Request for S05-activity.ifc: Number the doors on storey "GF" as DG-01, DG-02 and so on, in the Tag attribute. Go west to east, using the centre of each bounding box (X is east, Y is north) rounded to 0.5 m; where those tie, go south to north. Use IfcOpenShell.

First a look at what the model holds.

```python
import ifcopenshell
import ifcopenshell.util.element
import ifcopenshell.util.placement

model = ifcopenshell.open("S05-activity.ifc")
print(model.schema)
storey = next(s for s in model.by_type("IfcBuildingStorey") if s.Name == "GF")
doors = [e for e in ifcopenshell.util.element.get_decomposition(storey) if e.is_a("IfcDoor")]
for e in sorted(doors, key=lambda e: e.id()):
    origin = ifcopenshell.util.placement.get_local_placement(e.ObjectPlacement)[:3, 3]
    print(e.id(), e.Tag, e.Name, origin.round(2) + 0.0, sep=" | ")
```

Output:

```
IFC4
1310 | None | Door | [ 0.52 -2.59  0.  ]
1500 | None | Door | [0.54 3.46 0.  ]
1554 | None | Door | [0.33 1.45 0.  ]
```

```python
import ifcopenshell
import ifcopenshell.geom
import ifcopenshell.util.element
import ifcopenshell.util.shape

model = ifcopenshell.open("S05-activity.ifc")
settings = ifcopenshell.geom.settings()
settings.set("use-world-coords", True)


def centre(element):
    shape = ifcopenshell.geom.create_shape(settings, element)
    return ifcopenshell.util.shape.get_bbox_centroid(shape.geometry)


storey = next(s for s in model.by_type("IfcBuildingStorey") if s.Name == "GF")
doors = [e for e in ifcopenshell.util.element.get_decomposition(storey) if e.is_a("IfcDoor")]

# Insertion points can sit at a corner or the storey origin, so sort by the geometry (in metres).
centres = {e: centre(e) for e in doors}
doors.sort(key=lambda e: (round(centres[e][0] / 0.5), centres[e][1]))

for i, e in enumerate(doors, start=1):
    number = f"DG-{i:02d}"
    e.Tag = number
    print(e.id(), number)

model.write("S05-activity_updated.ifc")
```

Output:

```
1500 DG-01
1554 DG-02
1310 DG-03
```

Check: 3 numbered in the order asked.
